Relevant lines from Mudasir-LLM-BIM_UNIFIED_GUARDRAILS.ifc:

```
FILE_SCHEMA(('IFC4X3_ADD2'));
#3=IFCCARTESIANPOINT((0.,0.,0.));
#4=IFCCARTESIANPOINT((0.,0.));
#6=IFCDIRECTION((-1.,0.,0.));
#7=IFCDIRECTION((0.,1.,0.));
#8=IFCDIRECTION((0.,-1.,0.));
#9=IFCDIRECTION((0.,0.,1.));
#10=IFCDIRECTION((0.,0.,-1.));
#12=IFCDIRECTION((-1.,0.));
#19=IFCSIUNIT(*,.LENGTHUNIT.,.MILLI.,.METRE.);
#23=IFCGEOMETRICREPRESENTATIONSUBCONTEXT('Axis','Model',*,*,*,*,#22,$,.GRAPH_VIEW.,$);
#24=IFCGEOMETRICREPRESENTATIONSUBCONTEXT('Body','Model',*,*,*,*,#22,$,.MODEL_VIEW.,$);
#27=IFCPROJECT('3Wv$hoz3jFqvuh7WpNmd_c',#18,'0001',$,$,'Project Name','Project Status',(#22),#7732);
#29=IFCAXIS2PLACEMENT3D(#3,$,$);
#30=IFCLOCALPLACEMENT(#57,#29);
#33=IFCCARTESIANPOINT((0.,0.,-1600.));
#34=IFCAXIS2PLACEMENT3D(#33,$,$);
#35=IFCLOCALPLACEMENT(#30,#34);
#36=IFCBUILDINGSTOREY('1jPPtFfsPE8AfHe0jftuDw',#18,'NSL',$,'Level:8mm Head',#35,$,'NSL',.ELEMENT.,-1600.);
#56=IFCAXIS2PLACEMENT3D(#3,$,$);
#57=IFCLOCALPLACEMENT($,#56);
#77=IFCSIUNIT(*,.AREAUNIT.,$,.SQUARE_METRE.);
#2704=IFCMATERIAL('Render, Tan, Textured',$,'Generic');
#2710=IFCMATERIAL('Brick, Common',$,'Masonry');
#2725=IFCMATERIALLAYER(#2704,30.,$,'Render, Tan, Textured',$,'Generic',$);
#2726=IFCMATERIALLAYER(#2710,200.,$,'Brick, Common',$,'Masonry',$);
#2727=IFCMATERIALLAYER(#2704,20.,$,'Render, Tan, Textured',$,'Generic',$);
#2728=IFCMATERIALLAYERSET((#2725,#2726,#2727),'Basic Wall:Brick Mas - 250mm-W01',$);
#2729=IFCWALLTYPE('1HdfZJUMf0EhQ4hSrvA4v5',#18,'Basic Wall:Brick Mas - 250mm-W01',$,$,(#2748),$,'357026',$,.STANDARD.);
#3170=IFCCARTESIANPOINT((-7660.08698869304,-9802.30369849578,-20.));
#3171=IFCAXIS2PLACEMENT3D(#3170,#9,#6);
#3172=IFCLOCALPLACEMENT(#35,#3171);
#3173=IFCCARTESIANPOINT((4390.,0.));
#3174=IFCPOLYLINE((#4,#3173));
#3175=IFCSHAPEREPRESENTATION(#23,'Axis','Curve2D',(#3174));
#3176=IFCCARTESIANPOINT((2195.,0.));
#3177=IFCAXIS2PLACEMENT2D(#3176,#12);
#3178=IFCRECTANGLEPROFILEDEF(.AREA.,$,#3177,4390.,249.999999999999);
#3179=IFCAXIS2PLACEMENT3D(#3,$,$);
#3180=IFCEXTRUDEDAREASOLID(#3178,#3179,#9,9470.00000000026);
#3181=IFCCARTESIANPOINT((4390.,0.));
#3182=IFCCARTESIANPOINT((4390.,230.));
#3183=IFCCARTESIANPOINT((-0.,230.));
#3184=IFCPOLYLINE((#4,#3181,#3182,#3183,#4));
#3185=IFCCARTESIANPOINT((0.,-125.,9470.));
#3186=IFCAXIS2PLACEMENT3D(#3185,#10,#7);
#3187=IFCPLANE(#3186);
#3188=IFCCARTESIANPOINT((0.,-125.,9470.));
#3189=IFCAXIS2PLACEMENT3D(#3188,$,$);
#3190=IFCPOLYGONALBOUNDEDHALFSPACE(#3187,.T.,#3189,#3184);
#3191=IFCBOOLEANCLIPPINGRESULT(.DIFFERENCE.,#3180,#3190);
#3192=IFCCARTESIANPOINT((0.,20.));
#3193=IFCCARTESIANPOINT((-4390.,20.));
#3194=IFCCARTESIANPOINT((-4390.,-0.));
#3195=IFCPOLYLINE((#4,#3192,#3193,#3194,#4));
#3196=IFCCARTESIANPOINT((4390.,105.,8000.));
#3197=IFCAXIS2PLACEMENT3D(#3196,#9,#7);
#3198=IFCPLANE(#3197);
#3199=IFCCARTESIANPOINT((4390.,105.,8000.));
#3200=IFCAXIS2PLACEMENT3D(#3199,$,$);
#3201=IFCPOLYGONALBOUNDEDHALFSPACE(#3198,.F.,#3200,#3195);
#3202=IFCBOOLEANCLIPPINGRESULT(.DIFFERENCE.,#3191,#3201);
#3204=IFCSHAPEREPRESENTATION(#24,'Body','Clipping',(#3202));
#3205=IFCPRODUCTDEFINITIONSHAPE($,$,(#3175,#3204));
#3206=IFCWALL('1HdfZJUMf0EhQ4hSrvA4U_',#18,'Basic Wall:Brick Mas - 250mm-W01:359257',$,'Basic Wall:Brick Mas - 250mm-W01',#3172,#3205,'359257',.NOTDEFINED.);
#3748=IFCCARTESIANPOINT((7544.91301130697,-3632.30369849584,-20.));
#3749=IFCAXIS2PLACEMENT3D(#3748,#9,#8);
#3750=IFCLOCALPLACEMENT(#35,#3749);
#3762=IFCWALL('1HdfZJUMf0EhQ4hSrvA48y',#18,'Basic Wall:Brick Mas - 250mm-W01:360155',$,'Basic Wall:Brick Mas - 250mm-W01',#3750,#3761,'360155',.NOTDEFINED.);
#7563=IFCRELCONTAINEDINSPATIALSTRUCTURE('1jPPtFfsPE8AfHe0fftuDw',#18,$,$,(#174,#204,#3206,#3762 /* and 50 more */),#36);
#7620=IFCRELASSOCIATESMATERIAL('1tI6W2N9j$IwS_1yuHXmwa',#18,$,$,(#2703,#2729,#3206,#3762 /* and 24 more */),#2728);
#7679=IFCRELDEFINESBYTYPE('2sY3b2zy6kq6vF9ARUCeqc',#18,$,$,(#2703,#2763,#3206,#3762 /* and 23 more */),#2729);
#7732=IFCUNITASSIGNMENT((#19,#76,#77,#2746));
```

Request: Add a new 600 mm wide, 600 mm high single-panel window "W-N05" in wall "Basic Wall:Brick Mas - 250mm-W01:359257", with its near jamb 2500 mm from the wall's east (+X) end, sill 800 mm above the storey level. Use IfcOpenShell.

```python
import numpy as np
import ifcopenshell
import ifcopenshell.api.feature
import ifcopenshell.api.geometry
import ifcopenshell.api.root
import ifcopenshell.api.spatial
import ifcopenshell.geom
import ifcopenshell.util.element
import ifcopenshell.util.placement
import ifcopenshell.util.representation
import ifcopenshell.util.shape
import ifcopenshell.util.unit

model = ifcopenshell.open("Mudasir-LLM-BIM_UNIFIED_GUARDRAILS.ifc")
unit_scale = ifcopenshell.util.unit.calculate_unit_scale(model)
settings = ifcopenshell.geom.settings()


def volume(element):
    """Net volume in cubic metres, openings subtracted."""
    shape = ifcopenshell.geom.create_shape(settings, element)
    return ifcopenshell.util.shape.get_volume(shape.geometry)


wall = model.by_guid("1HdfZJUMf0EhQ4hSrvA4U_")
storey = ifcopenshell.util.element.get_container(wall, ifc_class="IfcBuildingStorey")
context = ifcopenshell.util.representation.get_context(model, "Model", "Body", "MODEL_VIEW")
before = volume(wall)

width, height, from_end, sill = 0.6, 0.6, 2.5, 0.8  # metres

# The wall runs along its own X axis, and the end named is its -X end.
wall_shape = ifcopenshell.geom.create_shape(settings, wall)
x, y, z = ifcopenshell.util.shape.get_vertices(wall_shape.geometry).T
start = x.min() + from_end
face, thickness = float(y.min()), float(y.max() - y.min())
wall_matrix = ifcopenshell.util.placement.get_local_placement(wall.ObjectPlacement)
level = ifcopenshell.util.placement.get_local_placement(storey.ObjectPlacement)[2, 3]


def in_wall(x, y):
    """Placement at x, y metres in the wall's axes, at sill height."""
    matrix = wall_matrix.copy()
    matrix[:, 3] = wall_matrix @ np.array([x / unit_scale, y / unit_scale, 0.0, 1.0])
    matrix[2, 3] = level + sill / unit_scale
    return matrix


# Opening: a box that overshoots both wall faces by 50 mm.
opening = ifcopenshell.api.root.create_entity(model, ifc_class="IfcOpeningElement", predefined_type="OPENING")
box = ifcopenshell.api.geometry.add_wall_representation(
    model, context=context, length=width, height=height, thickness=thickness + 0.1
)
ifcopenshell.api.geometry.assign_representation(model, product=opening, representation=box)
ifcopenshell.api.geometry.edit_object_placement(model, product=opening, matrix=in_wall(start, face - 0.05), is_si=False)
ifcopenshell.api.feature.add_feature(model, feature=opening, element=wall)

window = ifcopenshell.api.root.create_entity(model, ifc_class="IfcWindow", name="W-N05", predefined_type="WINDOW")
window.OverallWidth, window.OverallHeight = width / unit_scale, height / unit_scale
window.PartitioningType = "SINGLE_PANEL"
body = ifcopenshell.api.geometry.add_window_representation(
    model,
    context=context,
    overall_width=window.OverallWidth,
    overall_height=window.OverallHeight,
    partition_type="SINGLE_PANEL",
)
ifcopenshell.api.geometry.assign_representation(model, product=window, representation=body)
ifcopenshell.api.spatial.assign_container(model, products=[window], relating_structure=storey)
ifcopenshell.api.feature.add_filling(model, opening=opening, element=window)

# Centre the window in the wall's thickness.
ifcopenshell.api.geometry.edit_object_placement(model, product=window, matrix=in_wall(start, face), is_si=False)
window_shape = ifcopenshell.geom.create_shape(settings, window)
depth = ifcopenshell.util.shape.get_vertices(window_shape.geometry)[:, 1]
offset = face + thickness / 2 - (depth.min() + depth.max()) / 2
ifcopenshell.api.geometry.edit_object_placement(model, product=window, matrix=in_wall(start, offset), is_si=False)

after = volume(wall)

print(f"wall volume {before:.3f} -> {after:.3f} m3")

model.write("Mudasir-LLM-BIM_UNIFIED_GUARDRAILS_rev.ifc")
```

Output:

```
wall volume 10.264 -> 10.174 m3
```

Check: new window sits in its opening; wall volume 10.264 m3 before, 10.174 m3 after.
